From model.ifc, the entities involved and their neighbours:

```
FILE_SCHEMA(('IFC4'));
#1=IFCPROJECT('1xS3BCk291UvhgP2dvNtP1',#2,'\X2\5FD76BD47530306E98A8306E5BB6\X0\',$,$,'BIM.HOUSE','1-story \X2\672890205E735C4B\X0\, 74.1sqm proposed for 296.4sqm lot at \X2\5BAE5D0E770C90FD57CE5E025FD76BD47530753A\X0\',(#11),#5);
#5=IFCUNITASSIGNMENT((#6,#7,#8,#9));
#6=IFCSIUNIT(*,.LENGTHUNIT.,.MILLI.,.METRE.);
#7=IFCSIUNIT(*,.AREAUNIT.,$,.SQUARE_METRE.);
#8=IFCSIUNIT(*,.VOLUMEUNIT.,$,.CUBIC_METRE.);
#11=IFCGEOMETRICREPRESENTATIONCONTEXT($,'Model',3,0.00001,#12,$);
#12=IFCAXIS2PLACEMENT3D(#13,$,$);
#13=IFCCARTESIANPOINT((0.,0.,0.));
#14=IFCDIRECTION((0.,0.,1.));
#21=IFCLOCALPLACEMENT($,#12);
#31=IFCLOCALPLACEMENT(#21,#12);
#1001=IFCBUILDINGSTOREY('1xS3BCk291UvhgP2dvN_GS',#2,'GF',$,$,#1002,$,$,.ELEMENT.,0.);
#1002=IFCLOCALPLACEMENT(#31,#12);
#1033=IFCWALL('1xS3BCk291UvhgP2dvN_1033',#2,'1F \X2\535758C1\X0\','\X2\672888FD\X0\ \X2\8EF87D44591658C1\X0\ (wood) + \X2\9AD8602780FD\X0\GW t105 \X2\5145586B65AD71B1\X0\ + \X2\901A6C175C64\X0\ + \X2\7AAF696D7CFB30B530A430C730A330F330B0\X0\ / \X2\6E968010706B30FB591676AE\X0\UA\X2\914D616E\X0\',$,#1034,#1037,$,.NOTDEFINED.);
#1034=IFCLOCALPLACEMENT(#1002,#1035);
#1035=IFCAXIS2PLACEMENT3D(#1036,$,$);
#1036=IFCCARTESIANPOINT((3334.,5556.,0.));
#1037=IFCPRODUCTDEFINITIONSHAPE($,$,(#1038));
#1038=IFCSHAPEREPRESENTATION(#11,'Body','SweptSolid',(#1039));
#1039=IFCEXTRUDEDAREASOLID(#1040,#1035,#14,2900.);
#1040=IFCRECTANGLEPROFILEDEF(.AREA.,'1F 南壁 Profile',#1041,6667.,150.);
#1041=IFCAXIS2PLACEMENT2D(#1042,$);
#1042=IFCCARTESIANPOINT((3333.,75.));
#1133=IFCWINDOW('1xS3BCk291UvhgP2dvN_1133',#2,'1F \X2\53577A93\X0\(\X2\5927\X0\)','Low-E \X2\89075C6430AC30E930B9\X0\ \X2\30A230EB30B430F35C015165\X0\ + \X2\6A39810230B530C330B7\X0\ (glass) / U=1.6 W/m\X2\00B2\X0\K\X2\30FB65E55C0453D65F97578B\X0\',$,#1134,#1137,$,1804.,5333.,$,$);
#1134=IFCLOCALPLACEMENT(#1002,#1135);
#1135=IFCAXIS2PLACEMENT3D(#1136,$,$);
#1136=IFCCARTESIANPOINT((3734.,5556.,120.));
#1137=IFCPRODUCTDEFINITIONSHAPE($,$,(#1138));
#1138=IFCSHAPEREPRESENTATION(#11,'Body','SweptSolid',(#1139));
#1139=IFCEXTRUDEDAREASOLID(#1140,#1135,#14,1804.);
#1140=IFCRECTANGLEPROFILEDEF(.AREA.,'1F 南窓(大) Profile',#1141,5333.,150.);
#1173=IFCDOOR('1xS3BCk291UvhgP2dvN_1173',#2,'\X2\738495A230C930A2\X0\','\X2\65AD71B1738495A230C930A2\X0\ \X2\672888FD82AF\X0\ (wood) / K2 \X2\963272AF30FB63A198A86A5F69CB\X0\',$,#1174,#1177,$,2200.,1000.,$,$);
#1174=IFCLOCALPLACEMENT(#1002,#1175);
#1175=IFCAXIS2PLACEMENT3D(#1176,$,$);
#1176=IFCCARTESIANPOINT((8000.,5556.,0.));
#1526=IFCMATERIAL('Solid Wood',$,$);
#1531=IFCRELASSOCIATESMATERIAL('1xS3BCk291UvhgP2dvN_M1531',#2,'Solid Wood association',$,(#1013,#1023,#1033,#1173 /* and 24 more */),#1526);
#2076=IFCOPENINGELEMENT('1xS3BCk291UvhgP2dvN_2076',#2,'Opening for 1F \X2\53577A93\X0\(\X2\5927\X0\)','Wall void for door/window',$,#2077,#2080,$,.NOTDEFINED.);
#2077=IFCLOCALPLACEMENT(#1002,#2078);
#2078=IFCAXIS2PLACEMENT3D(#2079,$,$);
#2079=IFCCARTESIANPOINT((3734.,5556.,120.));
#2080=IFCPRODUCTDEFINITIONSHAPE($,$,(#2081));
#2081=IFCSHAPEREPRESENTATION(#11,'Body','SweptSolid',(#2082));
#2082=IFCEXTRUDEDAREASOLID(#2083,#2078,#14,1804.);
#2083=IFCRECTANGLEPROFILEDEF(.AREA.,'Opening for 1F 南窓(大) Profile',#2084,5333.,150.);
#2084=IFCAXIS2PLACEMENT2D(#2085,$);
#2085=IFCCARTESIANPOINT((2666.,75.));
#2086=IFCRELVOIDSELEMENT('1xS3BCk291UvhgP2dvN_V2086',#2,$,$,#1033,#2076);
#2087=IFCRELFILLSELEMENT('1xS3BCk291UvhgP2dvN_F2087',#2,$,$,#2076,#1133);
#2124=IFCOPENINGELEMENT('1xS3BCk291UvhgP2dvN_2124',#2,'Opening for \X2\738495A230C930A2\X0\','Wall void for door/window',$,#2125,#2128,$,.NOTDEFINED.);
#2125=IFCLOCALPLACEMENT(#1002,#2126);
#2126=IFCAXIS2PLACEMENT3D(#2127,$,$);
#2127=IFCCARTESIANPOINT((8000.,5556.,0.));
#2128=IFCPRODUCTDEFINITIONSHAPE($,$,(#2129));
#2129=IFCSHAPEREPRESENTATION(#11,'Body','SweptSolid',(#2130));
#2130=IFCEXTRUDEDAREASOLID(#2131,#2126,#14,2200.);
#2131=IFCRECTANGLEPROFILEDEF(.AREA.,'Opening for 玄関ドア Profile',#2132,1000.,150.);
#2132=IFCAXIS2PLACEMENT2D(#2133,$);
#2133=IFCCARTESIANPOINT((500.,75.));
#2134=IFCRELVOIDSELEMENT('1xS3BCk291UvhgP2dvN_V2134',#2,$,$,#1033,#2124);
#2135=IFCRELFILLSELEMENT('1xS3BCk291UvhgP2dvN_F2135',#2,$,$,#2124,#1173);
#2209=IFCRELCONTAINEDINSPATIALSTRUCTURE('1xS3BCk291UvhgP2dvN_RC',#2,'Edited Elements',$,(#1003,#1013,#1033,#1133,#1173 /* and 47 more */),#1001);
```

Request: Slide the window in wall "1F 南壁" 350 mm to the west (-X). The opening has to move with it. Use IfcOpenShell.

```python
import ifcopenshell
import ifcopenshell.api.geometry
import ifcopenshell.util.placement
import ifcopenshell.util.unit

model = ifcopenshell.open("model.ifc")
unit_scale = ifcopenshell.util.unit.calculate_unit_scale(model)

window = model.by_guid("1xS3BCk291UvhgP2dvN_1133")
opening = window.FillsVoids[0].RelatingOpeningElement
wall = opening.VoidsElements[0].RelatingBuildingElement

wall_matrix = ifcopenshell.util.placement.get_local_placement(wall.ObjectPlacement)
shift = wall_matrix[:3, 0] * -0.35 / unit_scale
before = ifcopenshell.util.placement.get_local_placement(window.ObjectPlacement)[:3, 3].copy()

# The window is not placed relative to its opening, so move both.
for product in (opening, window):
    matrix = ifcopenshell.util.placement.get_local_placement(product.ObjectPlacement)
    matrix[:3, 3] += shift
    ifcopenshell.api.geometry.edit_object_placement(model, product=product, matrix=matrix, is_si=False)

after = ifcopenshell.util.placement.get_local_placement(window.ObjectPlacement)[:3, 3]
print("window moved by", (after - before).round(3) + 0.0)

model.write("model_updated.ifc")
```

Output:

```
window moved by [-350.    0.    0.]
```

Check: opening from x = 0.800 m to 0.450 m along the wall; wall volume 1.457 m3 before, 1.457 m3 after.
